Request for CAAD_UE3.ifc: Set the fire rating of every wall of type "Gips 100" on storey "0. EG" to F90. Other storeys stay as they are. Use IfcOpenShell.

First a look at what the model holds.

```python
import ifcopenshell
import ifcopenshell.util.element

model = ifcopenshell.open("CAAD_UE3.ifc")
print(model.schema)
storey = next(s for s in model.by_type("IfcBuildingStorey") if s.Name == "0. EG")
walls = [e for e in ifcopenshell.util.element.get_decomposition(storey) if e.is_a("IfcWall")]
seen = {}
for e in walls:
    element_type = ifcopenshell.util.element.get_type(e)
    key = (element_type.Name if element_type != e and element_type else None, ifcopenshell.util.element.get_pset(e, "Pset_WallCommon", "FireRating"))
    seen[key] = seen.get(key, 0) + 1
for (name, value), count in sorted(seen.items(), key=str):
    print(count, "x", name, "|", value)
```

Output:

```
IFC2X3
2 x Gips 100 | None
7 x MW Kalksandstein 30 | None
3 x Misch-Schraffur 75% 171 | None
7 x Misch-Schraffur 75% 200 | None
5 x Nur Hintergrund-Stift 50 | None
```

```python
import ifcopenshell
import ifcopenshell.api.pset
import ifcopenshell.util.element

model = ifcopenshell.open("CAAD_UE3.ifc")

storey = next(s for s in model.by_type("IfcBuildingStorey") if s.Name == "0. EG")
walls = [e for e in ifcopenshell.util.element.get_decomposition(storey) if e.is_a("IfcWall")]

count = 0
for e in walls:
    element_type = ifcopenshell.util.element.get_type(e)
    if element_type in (None, e) or element_type.Name != "Gips 100":
        continue
    # add_pset returns the element's existing set when there is one.
    pset = ifcopenshell.api.pset.add_pset(model, product=e, name="Pset_WallCommon")
    ifcopenshell.api.pset.edit_pset(model, pset=pset, properties={"FireRating": "F90"})
    count += 1

print(count, "walls updated")

model.write("CAAD_UE3_rev.ifc")
```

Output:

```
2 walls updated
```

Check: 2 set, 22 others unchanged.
